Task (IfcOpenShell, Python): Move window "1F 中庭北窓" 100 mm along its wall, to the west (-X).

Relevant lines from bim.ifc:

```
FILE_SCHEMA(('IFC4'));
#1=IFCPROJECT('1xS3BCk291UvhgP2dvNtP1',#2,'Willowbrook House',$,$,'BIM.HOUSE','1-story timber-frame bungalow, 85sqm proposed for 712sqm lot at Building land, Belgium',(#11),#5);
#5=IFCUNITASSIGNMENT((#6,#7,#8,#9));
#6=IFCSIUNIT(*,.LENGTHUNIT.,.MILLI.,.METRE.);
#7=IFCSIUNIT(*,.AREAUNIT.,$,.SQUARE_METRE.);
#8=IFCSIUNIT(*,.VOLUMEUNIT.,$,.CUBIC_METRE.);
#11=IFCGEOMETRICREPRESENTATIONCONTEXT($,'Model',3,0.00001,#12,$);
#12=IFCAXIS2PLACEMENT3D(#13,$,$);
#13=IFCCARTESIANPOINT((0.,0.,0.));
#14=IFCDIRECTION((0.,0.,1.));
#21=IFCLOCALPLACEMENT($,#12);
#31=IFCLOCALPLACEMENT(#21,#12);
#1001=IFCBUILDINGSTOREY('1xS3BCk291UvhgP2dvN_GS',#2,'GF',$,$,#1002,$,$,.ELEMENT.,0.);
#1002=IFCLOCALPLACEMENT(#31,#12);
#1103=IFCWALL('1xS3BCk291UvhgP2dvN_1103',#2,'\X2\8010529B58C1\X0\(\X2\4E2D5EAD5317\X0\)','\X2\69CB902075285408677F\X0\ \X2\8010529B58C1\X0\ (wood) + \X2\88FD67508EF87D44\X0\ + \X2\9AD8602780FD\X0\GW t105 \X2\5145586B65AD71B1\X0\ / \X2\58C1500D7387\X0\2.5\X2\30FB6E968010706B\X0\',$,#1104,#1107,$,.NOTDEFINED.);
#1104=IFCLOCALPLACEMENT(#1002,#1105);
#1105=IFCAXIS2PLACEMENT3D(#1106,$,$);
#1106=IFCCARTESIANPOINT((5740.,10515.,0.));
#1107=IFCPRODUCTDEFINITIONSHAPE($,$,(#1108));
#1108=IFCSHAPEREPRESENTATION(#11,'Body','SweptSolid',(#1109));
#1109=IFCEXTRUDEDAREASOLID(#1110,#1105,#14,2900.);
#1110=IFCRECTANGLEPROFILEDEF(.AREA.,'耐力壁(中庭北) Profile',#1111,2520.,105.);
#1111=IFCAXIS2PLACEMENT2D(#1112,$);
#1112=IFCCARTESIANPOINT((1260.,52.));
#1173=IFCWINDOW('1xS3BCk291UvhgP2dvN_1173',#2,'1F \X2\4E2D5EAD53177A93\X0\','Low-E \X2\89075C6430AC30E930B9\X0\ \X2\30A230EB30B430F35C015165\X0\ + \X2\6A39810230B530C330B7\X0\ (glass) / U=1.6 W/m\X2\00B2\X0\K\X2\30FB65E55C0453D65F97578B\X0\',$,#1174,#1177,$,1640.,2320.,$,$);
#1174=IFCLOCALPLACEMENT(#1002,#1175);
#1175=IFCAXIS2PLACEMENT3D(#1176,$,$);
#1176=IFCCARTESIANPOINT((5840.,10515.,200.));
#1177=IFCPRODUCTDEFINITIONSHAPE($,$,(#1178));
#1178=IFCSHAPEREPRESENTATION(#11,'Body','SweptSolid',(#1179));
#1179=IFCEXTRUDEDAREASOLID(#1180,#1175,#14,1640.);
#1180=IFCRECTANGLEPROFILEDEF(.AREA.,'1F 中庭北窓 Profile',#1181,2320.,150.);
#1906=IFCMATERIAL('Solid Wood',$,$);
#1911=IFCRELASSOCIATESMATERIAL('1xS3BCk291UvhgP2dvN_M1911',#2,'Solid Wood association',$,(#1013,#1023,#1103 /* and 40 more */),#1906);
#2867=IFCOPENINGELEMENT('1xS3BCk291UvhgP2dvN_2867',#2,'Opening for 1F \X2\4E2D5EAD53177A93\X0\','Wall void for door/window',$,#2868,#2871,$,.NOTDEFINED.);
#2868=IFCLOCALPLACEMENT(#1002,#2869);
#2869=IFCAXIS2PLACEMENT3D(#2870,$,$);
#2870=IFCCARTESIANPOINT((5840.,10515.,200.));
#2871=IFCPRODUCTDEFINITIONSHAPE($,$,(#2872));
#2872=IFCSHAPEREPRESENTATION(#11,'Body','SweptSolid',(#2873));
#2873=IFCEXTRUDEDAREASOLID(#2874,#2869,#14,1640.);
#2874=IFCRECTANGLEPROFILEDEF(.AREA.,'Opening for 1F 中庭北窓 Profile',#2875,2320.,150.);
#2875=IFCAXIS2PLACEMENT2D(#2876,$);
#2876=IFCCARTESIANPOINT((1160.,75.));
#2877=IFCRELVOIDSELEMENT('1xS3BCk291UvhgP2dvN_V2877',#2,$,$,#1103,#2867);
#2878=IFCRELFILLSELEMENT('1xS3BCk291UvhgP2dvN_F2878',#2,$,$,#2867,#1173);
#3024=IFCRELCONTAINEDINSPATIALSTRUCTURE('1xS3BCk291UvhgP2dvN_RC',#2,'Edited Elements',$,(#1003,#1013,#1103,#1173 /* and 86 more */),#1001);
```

```python
import ifcopenshell
import ifcopenshell.api.geometry
import ifcopenshell.util.placement

model = ifcopenshell.open("bim.ifc")

window = model.by_id(1173)
opening = window.FillsVoids[0].RelatingOpeningElement
wall = opening.VoidsElements[0].RelatingBuildingElement

wall_matrix = ifcopenshell.util.placement.get_local_placement(wall.ObjectPlacement)
shift = wall_matrix[:3, 0] * -100.0
before = ifcopenshell.util.placement.get_local_placement(window.ObjectPlacement)[:3, 3].copy()

# The window is not placed relative to its opening, so move both.
for product in (opening, window):
    matrix = ifcopenshell.util.placement.get_local_placement(product.ObjectPlacement)
    matrix[:3, 3] += shift
    ifcopenshell.api.geometry.edit_object_placement(model, product=product, matrix=matrix, is_si=False)

after = ifcopenshell.util.placement.get_local_placement(window.ObjectPlacement)[:3, 3]
print("window moved by", (after - before).round(3) + 0.0)

model.write("bim_updated.ifc")
```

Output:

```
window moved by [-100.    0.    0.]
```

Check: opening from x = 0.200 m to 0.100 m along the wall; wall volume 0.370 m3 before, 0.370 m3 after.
